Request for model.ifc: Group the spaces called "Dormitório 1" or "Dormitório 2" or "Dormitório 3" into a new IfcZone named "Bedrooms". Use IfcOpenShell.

First a look at what the model holds.

```python
import ifcopenshell

model = ifcopenshell.open("model.ifc")
print(model.schema)
seen = {}
for space in model.by_type("IfcSpace"):
    seen[space.LongName] = seen.get(space.LongName, 0) + 1
for name, count in sorted(seen.items(), key=str):
    print(count, "x", name)
print("zones:", [z.Name for z in model.by_type("IfcZone")][:20])
```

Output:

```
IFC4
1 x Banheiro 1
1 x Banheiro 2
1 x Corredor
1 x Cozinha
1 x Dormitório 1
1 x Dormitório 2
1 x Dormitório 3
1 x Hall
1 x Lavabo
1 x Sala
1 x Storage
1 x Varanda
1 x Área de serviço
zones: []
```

```python
import ifcopenshell
import ifcopenshell.api.group
import ifcopenshell.api.root

model = ifcopenshell.open("model.ifc")

names = {"Dormitório 1", "Dormitório 2", "Dormitório 3"}
spaces = [s for s in model.by_type("IfcSpace") if s.LongName in names]

zone = ifcopenshell.api.root.create_entity(model, ifc_class="IfcZone", name="Bedrooms")
ifcopenshell.api.group.assign_group(model, products=spaces, group=zone)
print(len(spaces), "spaces in", zone.Name)

model.write("model_rev.ifc")
```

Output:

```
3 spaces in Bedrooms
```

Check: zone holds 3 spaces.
